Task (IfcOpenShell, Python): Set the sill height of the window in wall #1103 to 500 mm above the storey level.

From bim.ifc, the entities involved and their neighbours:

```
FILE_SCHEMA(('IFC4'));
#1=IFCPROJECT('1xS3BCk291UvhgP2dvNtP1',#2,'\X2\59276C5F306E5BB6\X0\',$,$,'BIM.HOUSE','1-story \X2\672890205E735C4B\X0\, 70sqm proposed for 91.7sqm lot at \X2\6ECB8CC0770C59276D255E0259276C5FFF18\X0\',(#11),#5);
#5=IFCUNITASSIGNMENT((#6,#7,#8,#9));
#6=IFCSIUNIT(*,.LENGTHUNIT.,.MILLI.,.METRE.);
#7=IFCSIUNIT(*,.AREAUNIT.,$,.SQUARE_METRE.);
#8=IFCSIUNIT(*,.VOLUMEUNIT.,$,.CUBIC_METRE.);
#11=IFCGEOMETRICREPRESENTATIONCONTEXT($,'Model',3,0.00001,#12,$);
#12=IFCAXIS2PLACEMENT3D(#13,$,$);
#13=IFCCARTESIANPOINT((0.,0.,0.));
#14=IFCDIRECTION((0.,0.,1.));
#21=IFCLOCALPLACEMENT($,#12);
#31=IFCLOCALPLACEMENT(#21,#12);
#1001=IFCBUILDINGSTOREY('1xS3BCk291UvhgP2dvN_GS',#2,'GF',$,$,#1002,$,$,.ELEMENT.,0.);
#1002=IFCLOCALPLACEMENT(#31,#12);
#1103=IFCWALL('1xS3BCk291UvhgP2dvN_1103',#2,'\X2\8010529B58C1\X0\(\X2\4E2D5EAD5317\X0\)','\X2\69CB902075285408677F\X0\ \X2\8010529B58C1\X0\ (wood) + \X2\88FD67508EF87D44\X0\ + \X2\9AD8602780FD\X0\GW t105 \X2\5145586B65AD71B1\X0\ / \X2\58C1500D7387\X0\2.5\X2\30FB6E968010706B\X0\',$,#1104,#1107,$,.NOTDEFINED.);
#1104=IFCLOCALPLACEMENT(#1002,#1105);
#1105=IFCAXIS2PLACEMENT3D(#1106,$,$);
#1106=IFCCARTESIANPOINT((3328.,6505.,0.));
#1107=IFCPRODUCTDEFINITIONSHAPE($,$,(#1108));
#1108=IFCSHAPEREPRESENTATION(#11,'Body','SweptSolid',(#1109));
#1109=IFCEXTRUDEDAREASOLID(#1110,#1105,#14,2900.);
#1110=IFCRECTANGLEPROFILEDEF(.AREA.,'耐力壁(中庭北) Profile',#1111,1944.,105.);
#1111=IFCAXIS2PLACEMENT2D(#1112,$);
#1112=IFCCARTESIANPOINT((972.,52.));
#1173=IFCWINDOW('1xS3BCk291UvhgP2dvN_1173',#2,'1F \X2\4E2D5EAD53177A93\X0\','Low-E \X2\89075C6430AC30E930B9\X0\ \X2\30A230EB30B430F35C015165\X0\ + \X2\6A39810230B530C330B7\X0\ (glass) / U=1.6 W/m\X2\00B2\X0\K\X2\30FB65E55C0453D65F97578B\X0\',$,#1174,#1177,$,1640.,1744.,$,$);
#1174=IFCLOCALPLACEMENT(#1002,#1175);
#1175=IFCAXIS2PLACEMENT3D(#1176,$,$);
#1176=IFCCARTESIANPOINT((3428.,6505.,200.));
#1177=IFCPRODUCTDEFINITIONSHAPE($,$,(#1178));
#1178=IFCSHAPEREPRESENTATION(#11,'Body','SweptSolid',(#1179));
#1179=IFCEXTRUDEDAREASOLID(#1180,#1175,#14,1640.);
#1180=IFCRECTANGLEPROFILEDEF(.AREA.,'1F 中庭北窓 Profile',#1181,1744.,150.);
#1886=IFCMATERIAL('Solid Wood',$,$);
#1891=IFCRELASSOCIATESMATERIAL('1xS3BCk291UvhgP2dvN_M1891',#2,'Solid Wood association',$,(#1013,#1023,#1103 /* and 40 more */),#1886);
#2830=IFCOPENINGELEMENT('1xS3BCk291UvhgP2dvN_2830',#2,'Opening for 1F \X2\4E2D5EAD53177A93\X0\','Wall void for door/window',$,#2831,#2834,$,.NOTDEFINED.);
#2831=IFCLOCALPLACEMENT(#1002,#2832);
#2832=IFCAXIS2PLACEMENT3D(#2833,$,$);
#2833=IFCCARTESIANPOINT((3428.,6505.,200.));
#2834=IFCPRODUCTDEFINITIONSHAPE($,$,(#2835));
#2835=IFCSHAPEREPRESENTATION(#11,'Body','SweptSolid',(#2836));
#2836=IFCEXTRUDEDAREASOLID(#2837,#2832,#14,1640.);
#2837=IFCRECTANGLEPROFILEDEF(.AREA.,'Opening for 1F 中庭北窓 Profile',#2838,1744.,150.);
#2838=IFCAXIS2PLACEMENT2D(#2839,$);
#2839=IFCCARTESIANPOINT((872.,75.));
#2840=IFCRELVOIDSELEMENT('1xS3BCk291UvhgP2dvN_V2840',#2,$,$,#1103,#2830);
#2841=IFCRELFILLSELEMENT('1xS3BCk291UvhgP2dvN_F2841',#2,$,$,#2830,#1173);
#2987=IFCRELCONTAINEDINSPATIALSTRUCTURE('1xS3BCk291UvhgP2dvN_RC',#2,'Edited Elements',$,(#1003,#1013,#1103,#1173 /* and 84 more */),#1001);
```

```python
import numpy as np
import ifcopenshell
import ifcopenshell.api.geometry
import ifcopenshell.geom
import ifcopenshell.util.element
import ifcopenshell.util.placement
import ifcopenshell.util.shape
import ifcopenshell.util.unit

model = ifcopenshell.open("bim.ifc")
unit_scale = ifcopenshell.util.unit.calculate_unit_scale(model)

window = model.by_guid("1xS3BCk291UvhgP2dvN_1173")
opening = window.FillsVoids[0].RelatingOpeningElement
storey = ifcopenshell.util.element.get_container(window, ifc_class="IfcBuildingStorey")
level = ifcopenshell.util.placement.get_local_placement(storey.ObjectPlacement)[2, 3]

# The opening's origin need not be at the sill, so measure its lowest point.
shape = ifcopenshell.geom.create_shape(ifcopenshell.geom.settings(), opening)
bottom = ifcopenshell.util.shape.get_shape_bottom_elevation(shape, shape.geometry) / unit_scale
dz = level + 500.0 - bottom

shift = np.array([0.0, 0.0, dz])
# The window is not placed relative to its opening, so move both.
for product in (opening, window):
    matrix = ifcopenshell.util.placement.get_local_placement(product.ObjectPlacement)
    matrix[:3, 3] += shift
    ifcopenshell.api.geometry.edit_object_placement(model, product=product, matrix=matrix, is_si=False)

print(f"moved by {dz * unit_scale:+.3f} m")

model.write("bim_edited.ifc")
```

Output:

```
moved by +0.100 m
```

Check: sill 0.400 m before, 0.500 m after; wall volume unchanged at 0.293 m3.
